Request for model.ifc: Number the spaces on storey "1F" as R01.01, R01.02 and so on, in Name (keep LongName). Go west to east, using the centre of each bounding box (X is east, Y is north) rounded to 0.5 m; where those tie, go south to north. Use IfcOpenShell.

First a look at what the model holds.

```python
import ifcopenshell
import ifcopenshell.util.element
import ifcopenshell.util.placement

model = ifcopenshell.open("model.ifc")
print(model.schema)
storey = next(s for s in model.by_type("IfcBuildingStorey") if s.Name == "1F")
spaces = [e for e in ifcopenshell.util.element.get_decomposition(storey) if e.is_a("IfcSpace")]
for e in sorted(spaces, key=lambda e: e.id()):
    origin = ifcopenshell.util.placement.get_local_placement(e.ObjectPlacement)[:3, 3]
    print(e.id(), e.Name, e.LongName, origin.round(2) + 0.0, sep=" | ")
```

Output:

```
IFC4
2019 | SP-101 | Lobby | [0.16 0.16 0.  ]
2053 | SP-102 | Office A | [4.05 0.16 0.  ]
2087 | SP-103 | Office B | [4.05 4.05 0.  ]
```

```python
import ifcopenshell
import ifcopenshell.geom
import ifcopenshell.util.element
import ifcopenshell.util.shape

model = ifcopenshell.open("model.ifc")
settings = ifcopenshell.geom.settings()
settings.set("use-world-coords", True)


def centre(element):
    shape = ifcopenshell.geom.create_shape(settings, element)
    return ifcopenshell.util.shape.get_bbox_centroid(shape.geometry)


storey = next(s for s in model.by_type("IfcBuildingStorey") if s.Name == "1F")
spaces = [e for e in ifcopenshell.util.element.get_decomposition(storey) if e.is_a("IfcSpace")]

# Insertion points can sit at a corner or the storey origin, so sort by the geometry (in metres).
centres = {e: centre(e) for e in spaces}
spaces.sort(key=lambda e: (round(centres[e][0] / 0.5), centres[e][1]))

for i, e in enumerate(spaces, start=1):
    number = f"R01.{i:02d}"
    e.Name = number
    print(e.id(), number)

model.write("model_edited.ifc")
```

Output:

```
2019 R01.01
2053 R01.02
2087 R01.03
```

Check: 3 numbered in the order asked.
